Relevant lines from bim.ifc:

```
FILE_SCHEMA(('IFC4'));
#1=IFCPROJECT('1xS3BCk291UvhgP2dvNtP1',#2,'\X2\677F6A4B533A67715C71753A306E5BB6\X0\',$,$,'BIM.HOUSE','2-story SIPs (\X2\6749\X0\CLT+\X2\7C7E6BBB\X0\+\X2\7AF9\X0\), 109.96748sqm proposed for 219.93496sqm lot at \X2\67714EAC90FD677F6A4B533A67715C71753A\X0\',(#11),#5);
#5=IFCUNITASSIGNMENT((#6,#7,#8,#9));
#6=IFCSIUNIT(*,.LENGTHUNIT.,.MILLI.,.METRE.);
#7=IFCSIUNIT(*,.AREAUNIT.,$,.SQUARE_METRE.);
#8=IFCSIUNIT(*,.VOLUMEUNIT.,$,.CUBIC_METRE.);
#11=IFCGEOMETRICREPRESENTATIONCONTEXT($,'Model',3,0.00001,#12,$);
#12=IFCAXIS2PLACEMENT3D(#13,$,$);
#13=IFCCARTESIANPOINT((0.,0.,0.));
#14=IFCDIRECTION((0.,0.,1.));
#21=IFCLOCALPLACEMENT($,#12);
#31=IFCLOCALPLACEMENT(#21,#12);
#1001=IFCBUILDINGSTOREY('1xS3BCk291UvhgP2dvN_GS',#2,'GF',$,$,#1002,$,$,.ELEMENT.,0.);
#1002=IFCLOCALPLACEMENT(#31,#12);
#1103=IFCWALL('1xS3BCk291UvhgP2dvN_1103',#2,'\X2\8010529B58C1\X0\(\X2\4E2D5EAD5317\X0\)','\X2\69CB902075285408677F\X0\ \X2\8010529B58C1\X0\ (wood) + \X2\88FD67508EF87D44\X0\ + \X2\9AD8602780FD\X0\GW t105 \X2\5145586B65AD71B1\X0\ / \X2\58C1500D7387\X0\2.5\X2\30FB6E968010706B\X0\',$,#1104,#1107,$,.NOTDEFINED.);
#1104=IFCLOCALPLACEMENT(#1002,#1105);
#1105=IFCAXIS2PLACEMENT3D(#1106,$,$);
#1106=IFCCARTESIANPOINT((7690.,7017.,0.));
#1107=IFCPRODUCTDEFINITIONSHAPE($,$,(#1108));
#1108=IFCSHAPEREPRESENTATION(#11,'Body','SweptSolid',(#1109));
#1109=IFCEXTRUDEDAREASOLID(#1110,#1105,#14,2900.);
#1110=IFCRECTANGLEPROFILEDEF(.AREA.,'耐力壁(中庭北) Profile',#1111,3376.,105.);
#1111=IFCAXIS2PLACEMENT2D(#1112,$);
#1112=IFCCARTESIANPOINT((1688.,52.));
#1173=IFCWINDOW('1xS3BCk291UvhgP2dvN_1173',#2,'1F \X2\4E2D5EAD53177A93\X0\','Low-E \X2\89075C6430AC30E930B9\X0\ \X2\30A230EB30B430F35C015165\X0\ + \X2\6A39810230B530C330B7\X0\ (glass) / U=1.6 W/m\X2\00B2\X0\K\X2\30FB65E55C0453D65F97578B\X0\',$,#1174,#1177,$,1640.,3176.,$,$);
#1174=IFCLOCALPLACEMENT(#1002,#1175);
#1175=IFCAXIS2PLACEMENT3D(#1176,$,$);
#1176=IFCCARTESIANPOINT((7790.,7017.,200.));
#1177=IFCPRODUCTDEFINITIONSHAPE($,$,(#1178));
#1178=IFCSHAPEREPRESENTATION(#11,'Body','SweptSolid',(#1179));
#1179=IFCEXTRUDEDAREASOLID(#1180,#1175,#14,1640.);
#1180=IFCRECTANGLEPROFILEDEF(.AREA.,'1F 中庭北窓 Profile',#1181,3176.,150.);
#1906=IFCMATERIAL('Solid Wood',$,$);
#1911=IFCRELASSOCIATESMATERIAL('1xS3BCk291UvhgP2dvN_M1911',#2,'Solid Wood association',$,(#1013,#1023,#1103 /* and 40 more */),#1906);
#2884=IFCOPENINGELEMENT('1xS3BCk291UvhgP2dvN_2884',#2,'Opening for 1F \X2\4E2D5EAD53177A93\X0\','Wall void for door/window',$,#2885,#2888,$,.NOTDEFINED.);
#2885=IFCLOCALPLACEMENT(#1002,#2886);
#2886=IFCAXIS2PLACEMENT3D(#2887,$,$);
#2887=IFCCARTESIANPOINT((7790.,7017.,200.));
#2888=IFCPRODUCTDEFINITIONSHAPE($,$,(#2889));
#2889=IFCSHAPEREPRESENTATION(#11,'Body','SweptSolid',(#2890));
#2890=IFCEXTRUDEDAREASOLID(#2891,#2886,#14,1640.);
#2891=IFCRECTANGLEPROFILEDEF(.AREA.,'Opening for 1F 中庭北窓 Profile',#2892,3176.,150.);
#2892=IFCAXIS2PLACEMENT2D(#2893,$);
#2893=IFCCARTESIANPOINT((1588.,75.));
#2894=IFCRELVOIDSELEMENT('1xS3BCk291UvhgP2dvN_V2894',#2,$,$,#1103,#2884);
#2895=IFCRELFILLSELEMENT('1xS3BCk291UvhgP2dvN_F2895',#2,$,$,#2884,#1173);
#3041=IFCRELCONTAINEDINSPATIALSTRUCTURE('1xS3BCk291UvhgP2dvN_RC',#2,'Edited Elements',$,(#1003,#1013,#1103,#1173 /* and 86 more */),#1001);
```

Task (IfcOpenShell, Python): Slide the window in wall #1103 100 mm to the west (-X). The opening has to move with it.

```python
import ifcopenshell
import ifcopenshell.api.geometry
import ifcopenshell.util.placement
import ifcopenshell.util.unit

model = ifcopenshell.open("bim.ifc")
unit_scale = ifcopenshell.util.unit.calculate_unit_scale(model)

window = model.by_guid("1xS3BCk291UvhgP2dvN_1173")
opening = window.FillsVoids[0].RelatingOpeningElement
wall = opening.VoidsElements[0].RelatingBuildingElement

wall_matrix = ifcopenshell.util.placement.get_local_placement(wall.ObjectPlacement)
shift = wall_matrix[:3, 0] * -0.1 / unit_scale
before = ifcopenshell.util.placement.get_local_placement(window.ObjectPlacement)[:3, 3].copy()

# The window is not placed relative to its opening, so move both.
for product in (opening, window):
    matrix = ifcopenshell.util.placement.get_local_placement(product.ObjectPlacement)
    matrix[:3, 3] += shift
    ifcopenshell.api.geometry.edit_object_placement(model, product=product, matrix=matrix, is_si=False)

after = ifcopenshell.util.placement.get_local_placement(window.ObjectPlacement)[:3, 3]
print("window moved by", (after - before).round(3) + 0.0)

model.write("bim_v2.ifc")
```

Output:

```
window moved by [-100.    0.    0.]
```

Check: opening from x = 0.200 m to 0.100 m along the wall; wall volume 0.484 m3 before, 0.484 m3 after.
